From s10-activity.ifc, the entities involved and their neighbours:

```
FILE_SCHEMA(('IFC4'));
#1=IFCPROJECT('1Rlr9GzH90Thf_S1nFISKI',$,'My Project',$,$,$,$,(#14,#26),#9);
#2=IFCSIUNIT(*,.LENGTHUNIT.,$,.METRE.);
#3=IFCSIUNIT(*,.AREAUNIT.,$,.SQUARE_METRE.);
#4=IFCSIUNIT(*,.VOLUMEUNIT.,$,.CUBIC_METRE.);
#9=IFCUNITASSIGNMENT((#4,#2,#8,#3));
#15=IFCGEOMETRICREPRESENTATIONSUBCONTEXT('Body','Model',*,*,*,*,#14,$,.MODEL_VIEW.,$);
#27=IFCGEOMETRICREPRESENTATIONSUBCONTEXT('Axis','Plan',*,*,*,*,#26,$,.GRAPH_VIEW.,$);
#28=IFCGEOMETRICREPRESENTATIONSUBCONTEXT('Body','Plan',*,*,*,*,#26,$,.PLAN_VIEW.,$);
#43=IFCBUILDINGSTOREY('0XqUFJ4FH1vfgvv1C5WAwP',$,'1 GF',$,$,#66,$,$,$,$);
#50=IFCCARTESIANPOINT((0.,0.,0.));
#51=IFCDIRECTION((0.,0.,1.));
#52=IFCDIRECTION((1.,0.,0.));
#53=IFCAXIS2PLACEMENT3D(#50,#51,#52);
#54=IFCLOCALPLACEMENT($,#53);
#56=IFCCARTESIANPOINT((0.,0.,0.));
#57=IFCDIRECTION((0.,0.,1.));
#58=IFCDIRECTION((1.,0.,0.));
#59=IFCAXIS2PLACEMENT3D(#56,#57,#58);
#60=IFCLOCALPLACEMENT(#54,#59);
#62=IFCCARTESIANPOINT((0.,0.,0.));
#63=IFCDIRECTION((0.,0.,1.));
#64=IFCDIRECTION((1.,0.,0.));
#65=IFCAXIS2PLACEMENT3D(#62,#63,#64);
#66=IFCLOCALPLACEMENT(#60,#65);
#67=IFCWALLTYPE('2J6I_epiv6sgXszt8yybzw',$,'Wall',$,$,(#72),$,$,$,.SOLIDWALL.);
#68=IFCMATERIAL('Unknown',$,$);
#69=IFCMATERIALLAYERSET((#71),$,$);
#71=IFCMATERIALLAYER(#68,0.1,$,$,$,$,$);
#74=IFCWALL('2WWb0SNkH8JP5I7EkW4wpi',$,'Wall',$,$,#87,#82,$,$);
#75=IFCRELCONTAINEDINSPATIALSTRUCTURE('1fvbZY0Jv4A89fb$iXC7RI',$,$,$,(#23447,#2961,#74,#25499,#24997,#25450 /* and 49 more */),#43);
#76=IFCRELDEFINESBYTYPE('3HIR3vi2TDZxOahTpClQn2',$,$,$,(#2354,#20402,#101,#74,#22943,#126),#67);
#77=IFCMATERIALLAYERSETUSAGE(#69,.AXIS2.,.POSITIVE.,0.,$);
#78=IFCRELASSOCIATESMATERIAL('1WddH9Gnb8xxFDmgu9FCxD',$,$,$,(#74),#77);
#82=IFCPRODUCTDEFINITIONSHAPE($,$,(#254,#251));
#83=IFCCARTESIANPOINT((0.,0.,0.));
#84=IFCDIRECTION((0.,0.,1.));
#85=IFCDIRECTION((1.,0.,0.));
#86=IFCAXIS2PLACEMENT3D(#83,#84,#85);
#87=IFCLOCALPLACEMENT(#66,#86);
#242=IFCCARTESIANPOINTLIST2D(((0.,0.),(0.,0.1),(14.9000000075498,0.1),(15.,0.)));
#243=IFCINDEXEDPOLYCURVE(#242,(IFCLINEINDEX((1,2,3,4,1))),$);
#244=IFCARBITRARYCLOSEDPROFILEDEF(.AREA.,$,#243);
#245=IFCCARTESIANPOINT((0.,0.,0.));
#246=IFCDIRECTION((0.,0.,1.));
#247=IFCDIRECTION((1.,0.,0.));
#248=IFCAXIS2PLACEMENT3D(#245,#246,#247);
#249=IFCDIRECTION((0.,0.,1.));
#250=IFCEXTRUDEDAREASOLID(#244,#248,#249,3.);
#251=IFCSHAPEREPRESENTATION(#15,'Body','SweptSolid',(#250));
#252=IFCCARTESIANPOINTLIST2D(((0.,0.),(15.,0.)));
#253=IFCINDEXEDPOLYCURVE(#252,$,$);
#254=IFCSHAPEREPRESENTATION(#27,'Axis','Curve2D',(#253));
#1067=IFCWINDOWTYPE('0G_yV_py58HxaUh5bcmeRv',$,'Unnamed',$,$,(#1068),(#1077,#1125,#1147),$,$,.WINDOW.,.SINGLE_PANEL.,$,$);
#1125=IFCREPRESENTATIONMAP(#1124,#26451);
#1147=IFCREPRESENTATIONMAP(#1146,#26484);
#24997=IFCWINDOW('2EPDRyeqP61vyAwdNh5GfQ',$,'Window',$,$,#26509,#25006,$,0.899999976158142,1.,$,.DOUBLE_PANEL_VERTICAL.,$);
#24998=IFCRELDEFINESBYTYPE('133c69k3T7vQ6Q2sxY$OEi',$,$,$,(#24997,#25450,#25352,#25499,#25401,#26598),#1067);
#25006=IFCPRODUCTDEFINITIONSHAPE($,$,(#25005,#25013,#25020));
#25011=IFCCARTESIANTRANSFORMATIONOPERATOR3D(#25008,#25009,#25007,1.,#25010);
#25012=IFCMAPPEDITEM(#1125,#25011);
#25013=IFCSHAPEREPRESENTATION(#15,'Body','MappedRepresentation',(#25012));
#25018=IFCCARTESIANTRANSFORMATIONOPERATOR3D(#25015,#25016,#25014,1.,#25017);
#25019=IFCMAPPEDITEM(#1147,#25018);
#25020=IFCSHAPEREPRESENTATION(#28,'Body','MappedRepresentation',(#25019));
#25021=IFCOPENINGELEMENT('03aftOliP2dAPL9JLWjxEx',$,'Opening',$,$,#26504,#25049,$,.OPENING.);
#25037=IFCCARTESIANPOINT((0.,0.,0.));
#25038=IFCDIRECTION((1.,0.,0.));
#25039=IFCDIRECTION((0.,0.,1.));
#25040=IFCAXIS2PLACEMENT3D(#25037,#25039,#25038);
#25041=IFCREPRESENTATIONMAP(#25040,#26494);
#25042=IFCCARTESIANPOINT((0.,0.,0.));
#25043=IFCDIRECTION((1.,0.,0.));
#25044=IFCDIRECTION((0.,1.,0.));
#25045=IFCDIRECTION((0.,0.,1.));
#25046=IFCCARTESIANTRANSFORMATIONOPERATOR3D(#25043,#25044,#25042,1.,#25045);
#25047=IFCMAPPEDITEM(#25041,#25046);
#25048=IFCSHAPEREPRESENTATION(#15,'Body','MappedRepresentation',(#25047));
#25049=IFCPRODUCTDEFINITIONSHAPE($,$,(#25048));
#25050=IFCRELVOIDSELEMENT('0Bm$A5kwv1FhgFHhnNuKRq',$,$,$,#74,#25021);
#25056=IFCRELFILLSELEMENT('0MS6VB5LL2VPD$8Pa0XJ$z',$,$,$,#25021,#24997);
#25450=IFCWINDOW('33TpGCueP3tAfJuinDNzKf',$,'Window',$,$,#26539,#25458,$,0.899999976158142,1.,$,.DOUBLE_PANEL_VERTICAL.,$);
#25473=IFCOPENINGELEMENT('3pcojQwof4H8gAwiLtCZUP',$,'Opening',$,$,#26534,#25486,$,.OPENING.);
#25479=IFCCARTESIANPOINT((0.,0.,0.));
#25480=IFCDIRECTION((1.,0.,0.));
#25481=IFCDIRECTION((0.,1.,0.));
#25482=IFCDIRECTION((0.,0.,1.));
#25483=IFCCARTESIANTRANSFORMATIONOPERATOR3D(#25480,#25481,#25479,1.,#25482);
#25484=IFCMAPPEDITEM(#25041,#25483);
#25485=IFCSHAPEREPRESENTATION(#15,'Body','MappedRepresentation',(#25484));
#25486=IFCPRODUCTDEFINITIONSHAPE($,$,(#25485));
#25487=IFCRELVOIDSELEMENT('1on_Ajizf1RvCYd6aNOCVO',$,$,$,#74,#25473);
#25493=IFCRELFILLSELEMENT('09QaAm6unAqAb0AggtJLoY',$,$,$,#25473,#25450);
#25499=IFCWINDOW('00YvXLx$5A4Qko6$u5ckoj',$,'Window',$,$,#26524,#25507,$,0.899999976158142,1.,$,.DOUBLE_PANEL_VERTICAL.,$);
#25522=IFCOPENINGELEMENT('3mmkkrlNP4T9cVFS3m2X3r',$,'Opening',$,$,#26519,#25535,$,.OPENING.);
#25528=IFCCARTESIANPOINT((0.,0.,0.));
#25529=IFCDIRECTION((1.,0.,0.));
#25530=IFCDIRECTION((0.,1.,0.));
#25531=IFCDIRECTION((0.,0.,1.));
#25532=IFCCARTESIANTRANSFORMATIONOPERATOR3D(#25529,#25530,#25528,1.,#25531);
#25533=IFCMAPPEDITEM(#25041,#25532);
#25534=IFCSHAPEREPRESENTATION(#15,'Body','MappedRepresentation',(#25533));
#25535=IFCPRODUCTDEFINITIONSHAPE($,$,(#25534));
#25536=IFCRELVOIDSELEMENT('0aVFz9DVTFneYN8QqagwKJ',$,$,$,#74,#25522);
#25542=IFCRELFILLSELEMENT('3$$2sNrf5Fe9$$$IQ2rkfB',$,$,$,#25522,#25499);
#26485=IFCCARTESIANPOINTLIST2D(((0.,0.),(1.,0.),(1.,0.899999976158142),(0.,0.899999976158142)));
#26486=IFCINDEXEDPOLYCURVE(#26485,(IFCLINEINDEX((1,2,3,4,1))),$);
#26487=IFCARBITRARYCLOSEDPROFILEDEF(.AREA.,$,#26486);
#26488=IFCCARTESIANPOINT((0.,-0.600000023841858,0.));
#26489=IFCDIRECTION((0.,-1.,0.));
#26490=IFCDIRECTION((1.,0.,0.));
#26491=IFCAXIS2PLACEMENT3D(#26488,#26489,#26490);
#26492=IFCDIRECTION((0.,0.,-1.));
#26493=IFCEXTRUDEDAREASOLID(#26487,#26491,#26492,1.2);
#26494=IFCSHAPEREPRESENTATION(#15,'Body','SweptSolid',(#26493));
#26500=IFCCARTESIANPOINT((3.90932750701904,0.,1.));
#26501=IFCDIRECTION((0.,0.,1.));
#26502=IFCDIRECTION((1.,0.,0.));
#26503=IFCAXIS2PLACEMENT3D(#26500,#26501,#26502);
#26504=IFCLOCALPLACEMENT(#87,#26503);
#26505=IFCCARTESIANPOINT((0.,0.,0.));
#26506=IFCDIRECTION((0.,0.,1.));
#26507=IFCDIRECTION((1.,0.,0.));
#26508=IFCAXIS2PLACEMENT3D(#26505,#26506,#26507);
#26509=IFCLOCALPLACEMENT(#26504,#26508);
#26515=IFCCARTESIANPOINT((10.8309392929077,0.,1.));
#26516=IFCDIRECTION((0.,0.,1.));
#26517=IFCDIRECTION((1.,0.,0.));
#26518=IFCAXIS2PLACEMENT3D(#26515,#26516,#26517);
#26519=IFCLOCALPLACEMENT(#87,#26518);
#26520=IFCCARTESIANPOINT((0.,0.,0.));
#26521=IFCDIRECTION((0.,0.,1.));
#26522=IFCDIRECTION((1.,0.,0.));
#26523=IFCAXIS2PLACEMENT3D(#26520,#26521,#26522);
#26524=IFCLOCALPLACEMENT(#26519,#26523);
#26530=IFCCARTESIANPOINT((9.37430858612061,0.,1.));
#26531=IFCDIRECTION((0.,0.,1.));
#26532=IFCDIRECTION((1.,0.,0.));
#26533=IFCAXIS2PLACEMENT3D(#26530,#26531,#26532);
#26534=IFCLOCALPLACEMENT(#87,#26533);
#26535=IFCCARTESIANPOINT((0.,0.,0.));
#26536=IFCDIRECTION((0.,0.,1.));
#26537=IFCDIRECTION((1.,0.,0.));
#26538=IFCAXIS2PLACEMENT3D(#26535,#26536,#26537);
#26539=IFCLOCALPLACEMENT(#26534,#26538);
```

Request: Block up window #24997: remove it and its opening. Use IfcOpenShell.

```python
import ifcopenshell
import ifcopenshell.api.feature
import ifcopenshell.api.root
import ifcopenshell.geom
import ifcopenshell.util.shape

model = ifcopenshell.open("s10-activity.ifc")
settings = ifcopenshell.geom.settings()


def volume(element):
    """Net volume in cubic metres, openings subtracted."""
    shape = ifcopenshell.geom.create_shape(settings, element)
    return ifcopenshell.util.shape.get_volume(shape.geometry)


window = model.by_guid("2EPDRyeqP61vyAwdNh5GfQ")
opening = window.FillsVoids[0].RelatingOpeningElement
wall = opening.VoidsElements[0].RelatingBuildingElement
before = volume(wall)

ifcopenshell.api.root.remove_product(model, product=window)
ifcopenshell.api.feature.remove_feature(model, feature=opening)

after = volume(wall)

print(f"wall volume {before:.3f} -> {after:.3f} m3")

model.write("s10-activity_v2.ifc")
```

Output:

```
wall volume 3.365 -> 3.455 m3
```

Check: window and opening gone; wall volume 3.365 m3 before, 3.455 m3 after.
